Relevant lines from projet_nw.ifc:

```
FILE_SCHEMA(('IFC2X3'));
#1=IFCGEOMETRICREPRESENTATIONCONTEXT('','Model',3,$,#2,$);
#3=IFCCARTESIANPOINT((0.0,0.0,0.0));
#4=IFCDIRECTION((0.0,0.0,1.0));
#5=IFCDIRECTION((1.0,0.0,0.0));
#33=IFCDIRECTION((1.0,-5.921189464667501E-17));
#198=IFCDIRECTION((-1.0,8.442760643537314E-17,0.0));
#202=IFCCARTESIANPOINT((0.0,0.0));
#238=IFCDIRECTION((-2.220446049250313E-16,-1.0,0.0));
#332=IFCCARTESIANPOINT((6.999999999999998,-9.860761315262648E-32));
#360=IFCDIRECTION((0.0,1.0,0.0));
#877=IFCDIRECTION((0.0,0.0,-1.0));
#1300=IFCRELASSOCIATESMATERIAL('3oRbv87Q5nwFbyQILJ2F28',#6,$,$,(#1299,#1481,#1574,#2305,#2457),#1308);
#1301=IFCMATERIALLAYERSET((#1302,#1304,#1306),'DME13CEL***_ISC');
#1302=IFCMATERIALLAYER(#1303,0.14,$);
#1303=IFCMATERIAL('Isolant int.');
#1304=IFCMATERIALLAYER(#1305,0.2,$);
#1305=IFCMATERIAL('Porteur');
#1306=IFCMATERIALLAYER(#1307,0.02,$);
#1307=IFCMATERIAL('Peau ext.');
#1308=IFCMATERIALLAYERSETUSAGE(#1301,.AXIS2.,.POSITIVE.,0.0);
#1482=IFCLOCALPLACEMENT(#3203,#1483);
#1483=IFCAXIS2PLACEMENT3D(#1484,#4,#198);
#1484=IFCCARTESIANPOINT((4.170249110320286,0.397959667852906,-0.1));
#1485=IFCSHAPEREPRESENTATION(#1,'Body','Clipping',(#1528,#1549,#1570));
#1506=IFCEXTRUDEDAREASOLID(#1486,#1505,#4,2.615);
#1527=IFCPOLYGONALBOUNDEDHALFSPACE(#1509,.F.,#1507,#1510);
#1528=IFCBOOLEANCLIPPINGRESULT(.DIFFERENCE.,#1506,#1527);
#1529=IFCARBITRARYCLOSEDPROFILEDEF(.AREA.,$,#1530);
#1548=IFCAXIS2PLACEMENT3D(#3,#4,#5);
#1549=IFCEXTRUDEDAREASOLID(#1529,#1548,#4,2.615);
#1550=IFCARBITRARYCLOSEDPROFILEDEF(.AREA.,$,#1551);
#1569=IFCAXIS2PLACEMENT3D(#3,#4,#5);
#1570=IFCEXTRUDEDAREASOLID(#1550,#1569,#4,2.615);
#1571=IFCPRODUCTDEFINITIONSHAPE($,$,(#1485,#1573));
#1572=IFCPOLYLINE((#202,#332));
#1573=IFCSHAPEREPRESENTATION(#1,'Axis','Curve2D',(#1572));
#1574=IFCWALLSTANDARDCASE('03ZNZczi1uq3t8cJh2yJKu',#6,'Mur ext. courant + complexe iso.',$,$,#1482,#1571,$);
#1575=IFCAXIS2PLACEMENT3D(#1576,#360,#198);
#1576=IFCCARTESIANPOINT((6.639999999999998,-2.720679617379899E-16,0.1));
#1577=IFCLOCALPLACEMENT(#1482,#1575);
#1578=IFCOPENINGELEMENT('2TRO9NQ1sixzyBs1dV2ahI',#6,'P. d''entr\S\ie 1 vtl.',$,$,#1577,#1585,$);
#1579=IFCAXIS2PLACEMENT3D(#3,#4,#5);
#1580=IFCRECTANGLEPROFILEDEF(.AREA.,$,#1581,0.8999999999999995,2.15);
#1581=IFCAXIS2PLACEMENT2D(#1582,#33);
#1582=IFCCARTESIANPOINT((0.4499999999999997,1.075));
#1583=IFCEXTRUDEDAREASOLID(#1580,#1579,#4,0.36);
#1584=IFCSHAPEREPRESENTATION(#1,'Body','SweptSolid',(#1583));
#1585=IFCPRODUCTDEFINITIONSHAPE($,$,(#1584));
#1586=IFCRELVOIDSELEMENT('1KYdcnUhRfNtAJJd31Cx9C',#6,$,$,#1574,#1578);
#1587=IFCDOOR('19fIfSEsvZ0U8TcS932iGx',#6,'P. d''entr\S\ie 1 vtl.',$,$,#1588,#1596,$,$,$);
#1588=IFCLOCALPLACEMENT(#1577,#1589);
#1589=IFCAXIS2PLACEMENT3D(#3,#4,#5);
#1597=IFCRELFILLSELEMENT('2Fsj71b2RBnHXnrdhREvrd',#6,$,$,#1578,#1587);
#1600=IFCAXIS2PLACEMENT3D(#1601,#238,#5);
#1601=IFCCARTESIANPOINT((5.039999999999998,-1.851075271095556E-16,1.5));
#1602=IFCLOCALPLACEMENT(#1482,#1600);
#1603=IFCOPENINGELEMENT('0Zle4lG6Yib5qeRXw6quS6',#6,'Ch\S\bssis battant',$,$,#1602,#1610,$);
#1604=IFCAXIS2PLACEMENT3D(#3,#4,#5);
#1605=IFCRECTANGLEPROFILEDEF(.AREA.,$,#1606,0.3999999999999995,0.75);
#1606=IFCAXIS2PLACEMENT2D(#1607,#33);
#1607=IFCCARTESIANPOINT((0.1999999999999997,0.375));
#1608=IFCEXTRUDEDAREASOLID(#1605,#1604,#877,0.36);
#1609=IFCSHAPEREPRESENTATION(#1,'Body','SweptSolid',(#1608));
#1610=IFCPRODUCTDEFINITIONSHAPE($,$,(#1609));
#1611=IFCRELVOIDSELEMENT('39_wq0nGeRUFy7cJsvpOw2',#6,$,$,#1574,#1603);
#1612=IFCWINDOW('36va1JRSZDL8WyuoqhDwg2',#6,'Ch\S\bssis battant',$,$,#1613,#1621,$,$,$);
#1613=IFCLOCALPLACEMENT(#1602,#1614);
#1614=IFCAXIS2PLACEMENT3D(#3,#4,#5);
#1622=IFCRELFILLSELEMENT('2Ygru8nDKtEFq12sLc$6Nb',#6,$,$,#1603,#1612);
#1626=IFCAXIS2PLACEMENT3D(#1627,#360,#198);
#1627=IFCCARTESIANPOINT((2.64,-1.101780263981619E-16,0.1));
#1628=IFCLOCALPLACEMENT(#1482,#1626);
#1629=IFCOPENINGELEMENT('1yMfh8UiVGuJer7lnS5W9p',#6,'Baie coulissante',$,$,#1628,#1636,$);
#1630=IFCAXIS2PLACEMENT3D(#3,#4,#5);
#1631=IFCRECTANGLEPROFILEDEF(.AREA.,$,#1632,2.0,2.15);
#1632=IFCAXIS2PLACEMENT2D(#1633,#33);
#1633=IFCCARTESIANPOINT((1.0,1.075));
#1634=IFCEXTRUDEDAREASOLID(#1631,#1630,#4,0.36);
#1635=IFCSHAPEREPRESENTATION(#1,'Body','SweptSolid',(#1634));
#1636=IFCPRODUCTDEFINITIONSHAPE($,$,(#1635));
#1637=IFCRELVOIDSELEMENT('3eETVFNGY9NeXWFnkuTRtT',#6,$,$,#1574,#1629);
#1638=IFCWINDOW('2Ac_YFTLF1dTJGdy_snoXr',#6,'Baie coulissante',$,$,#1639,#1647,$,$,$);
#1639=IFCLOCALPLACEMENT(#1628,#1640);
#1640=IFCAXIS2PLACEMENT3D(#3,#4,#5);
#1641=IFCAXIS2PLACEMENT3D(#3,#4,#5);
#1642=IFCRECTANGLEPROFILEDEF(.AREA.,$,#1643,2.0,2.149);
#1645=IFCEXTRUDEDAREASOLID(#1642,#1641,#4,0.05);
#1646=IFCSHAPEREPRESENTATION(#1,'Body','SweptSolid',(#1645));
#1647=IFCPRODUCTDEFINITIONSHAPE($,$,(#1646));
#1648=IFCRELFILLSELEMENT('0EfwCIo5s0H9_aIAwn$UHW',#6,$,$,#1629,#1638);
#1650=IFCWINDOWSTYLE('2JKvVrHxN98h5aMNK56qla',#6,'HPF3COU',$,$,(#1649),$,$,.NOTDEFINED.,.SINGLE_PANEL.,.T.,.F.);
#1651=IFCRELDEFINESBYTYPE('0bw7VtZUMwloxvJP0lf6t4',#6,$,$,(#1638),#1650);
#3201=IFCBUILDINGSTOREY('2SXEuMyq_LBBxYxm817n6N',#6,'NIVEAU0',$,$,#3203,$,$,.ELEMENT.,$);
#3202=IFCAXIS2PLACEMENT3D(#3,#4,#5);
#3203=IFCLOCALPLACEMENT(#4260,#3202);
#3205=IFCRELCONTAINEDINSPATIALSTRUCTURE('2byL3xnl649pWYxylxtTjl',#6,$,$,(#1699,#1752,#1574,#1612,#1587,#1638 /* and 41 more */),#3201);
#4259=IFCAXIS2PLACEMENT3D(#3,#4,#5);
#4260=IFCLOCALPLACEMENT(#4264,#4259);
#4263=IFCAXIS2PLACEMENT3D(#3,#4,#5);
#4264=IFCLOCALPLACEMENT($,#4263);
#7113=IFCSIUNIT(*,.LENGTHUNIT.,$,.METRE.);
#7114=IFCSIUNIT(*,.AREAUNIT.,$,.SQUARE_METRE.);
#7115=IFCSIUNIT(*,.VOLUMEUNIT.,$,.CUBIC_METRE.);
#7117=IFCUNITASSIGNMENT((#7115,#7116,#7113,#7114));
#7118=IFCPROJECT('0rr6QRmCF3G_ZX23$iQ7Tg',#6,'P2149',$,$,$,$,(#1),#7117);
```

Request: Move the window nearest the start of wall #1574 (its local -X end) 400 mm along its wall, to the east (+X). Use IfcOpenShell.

```python
import ifcopenshell
import ifcopenshell.api.geometry
import ifcopenshell.util.placement
import ifcopenshell.util.unit

model = ifcopenshell.open("projet_nw.ifc")
unit_scale = ifcopenshell.util.unit.calculate_unit_scale(model)

window = model.by_id(1638)
opening = window.FillsVoids[0].RelatingOpeningElement
wall = opening.VoidsElements[0].RelatingBuildingElement

wall_matrix = ifcopenshell.util.placement.get_local_placement(wall.ObjectPlacement)
shift = wall_matrix[:3, 0] * -0.4 / unit_scale
before = ifcopenshell.util.placement.get_local_placement(window.ObjectPlacement)[:3, 3].copy()

# The window is placed relative to its opening, so it follows when the opening moves.
matrix = ifcopenshell.util.placement.get_local_placement(opening.ObjectPlacement)
matrix[:3, 3] += shift
ifcopenshell.api.geometry.edit_object_placement(
    model, product=opening, matrix=matrix, is_si=False, should_transform_children=True
)

after = ifcopenshell.util.placement.get_local_placement(window.ObjectPlacement)[:3, 3]
print("window moved by", (after - before).round(3) + 0.0)

model.write("projet_nw-out.ifc")
```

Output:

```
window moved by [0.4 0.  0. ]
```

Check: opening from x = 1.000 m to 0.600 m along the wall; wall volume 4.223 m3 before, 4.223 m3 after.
